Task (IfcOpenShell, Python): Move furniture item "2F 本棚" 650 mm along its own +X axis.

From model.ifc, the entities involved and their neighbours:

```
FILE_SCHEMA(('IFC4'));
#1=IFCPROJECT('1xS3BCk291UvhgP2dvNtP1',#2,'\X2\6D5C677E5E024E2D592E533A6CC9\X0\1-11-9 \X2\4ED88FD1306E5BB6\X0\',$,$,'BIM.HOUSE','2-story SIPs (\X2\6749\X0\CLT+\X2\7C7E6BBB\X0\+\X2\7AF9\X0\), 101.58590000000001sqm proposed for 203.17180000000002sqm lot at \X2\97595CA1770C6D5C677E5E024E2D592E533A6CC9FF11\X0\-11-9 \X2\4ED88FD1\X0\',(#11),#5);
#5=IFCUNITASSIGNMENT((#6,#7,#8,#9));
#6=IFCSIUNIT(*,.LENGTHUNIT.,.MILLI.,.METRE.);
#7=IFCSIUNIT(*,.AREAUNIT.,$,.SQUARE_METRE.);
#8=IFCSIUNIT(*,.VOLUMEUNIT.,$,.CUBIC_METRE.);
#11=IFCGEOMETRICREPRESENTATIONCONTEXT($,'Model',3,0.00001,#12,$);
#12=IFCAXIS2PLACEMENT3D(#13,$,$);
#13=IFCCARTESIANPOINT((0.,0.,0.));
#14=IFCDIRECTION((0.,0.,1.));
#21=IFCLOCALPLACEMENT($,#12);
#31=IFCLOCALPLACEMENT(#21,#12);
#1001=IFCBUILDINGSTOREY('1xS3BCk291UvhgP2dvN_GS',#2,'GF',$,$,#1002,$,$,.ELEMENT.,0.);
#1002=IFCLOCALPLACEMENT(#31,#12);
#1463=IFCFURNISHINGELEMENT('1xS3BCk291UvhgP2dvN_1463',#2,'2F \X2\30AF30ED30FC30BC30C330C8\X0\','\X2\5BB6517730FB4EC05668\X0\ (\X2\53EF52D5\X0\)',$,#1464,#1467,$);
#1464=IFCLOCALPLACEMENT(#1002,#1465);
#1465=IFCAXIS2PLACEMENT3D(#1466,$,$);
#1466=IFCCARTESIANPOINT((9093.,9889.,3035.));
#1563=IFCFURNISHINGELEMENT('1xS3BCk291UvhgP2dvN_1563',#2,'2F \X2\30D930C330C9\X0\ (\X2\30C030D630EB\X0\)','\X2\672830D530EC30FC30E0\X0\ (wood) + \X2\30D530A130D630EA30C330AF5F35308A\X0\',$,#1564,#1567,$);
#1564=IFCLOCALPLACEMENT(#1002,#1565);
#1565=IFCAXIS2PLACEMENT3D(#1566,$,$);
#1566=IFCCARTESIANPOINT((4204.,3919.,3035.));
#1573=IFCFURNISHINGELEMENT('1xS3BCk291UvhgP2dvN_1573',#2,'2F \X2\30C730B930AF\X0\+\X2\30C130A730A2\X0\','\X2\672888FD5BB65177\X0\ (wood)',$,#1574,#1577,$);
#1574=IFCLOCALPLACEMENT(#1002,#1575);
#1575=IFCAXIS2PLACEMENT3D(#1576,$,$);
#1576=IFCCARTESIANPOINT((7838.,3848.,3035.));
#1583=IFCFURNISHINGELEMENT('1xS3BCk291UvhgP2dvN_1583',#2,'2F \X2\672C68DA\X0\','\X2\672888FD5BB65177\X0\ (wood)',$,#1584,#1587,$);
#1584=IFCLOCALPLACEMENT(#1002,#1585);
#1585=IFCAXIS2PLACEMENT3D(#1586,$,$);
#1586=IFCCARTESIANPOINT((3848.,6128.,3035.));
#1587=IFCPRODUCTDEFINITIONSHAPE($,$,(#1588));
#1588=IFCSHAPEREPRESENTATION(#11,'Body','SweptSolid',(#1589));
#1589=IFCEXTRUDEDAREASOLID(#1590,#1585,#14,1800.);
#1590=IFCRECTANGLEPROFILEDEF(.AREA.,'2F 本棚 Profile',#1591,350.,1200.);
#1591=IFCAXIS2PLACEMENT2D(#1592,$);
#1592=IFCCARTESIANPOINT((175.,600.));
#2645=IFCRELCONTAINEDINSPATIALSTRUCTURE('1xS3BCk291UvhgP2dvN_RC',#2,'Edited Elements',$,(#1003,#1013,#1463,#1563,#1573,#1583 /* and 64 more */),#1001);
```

```python
import ifcopenshell
import ifcopenshell.api.geometry
import ifcopenshell.util.placement
import ifcopenshell.util.unit

model = ifcopenshell.open("model.ifc")
unit_scale = ifcopenshell.util.unit.calculate_unit_scale(model)

item = model.by_id(1583)
matrix = ifcopenshell.util.placement.get_local_placement(item.ObjectPlacement)
matrix[:3, 3] += matrix[:3, 0] * 0.65 / unit_scale
ifcopenshell.api.geometry.edit_object_placement(model, product=item, matrix=matrix, is_si=False)

print(ifcopenshell.util.placement.get_local_placement(item.ObjectPlacement).round(3) + 0.0)

model.write("model_v2.ifc")
```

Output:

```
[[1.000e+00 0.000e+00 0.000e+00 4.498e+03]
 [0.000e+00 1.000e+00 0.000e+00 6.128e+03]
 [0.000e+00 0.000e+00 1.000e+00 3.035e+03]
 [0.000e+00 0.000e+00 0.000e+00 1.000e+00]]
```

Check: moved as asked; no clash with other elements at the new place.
